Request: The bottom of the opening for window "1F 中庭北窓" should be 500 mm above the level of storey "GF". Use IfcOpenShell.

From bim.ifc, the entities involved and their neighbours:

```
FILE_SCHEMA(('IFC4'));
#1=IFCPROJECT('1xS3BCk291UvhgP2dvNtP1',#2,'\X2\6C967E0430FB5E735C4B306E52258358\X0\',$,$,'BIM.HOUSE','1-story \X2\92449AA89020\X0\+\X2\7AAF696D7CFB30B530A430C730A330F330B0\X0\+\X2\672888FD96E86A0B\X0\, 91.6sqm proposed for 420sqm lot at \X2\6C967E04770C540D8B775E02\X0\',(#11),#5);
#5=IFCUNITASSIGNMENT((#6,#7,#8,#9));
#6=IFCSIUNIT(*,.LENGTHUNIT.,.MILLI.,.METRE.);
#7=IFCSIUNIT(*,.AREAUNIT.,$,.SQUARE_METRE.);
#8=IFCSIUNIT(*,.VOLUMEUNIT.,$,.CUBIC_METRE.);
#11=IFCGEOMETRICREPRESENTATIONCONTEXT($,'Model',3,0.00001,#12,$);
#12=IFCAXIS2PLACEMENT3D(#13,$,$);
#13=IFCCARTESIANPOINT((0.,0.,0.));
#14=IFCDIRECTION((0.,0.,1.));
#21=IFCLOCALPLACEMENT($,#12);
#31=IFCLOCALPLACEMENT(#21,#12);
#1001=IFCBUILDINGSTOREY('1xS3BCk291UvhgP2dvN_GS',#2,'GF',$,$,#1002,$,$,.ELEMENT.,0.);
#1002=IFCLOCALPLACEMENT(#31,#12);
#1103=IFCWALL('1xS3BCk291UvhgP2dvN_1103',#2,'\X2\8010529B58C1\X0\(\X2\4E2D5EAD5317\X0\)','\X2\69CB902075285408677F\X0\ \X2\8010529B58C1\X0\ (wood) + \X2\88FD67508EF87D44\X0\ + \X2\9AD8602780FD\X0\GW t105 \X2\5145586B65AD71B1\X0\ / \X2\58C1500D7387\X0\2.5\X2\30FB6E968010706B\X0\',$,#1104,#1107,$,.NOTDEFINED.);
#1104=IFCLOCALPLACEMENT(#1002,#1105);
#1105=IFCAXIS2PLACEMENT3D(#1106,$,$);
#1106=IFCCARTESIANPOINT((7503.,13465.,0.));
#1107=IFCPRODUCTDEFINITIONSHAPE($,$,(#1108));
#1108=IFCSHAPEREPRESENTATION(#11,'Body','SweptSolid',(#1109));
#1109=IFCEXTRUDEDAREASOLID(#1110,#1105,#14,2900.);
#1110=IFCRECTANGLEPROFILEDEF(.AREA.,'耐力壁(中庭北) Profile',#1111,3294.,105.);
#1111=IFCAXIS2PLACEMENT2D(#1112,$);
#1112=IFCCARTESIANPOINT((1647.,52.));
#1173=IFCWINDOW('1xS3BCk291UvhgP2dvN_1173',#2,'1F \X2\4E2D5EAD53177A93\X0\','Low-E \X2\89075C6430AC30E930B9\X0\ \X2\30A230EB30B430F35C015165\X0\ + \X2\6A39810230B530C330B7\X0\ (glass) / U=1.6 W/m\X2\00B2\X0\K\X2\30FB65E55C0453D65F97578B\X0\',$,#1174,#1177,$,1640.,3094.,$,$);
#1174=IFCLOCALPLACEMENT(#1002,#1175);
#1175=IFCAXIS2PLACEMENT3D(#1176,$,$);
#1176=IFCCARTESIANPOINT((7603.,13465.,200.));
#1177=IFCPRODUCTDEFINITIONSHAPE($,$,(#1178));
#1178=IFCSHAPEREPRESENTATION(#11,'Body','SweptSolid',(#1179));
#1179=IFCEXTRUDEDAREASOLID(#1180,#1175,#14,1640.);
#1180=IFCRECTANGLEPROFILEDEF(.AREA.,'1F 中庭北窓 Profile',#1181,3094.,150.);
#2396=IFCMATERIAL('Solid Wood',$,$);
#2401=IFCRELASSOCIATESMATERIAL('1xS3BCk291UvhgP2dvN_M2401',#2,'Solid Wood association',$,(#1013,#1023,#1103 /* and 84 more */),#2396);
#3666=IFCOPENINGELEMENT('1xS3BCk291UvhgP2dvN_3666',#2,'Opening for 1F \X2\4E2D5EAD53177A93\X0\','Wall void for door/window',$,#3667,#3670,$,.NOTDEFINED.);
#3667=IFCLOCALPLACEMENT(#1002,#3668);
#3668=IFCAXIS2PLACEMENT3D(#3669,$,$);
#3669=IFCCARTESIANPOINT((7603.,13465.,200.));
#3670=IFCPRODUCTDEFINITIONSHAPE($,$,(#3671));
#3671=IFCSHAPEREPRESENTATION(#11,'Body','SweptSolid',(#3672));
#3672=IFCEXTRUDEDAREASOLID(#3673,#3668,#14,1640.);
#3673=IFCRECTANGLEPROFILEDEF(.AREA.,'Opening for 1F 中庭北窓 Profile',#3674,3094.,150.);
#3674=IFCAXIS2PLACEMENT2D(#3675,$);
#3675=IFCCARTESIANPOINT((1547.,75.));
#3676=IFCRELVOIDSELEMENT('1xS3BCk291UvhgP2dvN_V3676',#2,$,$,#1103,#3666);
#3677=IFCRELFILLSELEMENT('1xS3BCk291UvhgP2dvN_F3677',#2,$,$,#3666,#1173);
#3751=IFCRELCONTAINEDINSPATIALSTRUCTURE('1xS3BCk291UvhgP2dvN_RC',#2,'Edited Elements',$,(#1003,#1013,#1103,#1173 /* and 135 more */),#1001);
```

```python
import numpy as np
import ifcopenshell
import ifcopenshell.api.geometry
import ifcopenshell.geom
import ifcopenshell.util.element
import ifcopenshell.util.placement
import ifcopenshell.util.shape
import ifcopenshell.util.unit

model = ifcopenshell.open("bim.ifc")
unit_scale = ifcopenshell.util.unit.calculate_unit_scale(model)

window = model.by_guid("1xS3BCk291UvhgP2dvN_1173")
opening = window.FillsVoids[0].RelatingOpeningElement
storey = ifcopenshell.util.element.get_container(window, ifc_class="IfcBuildingStorey")
level = ifcopenshell.util.placement.get_local_placement(storey.ObjectPlacement)[2, 3]

# The opening's origin need not be at the sill, so measure its lowest point.
shape = ifcopenshell.geom.create_shape(ifcopenshell.geom.settings(), opening)
bottom = ifcopenshell.util.shape.get_shape_bottom_elevation(shape, shape.geometry) / unit_scale
dz = level + 500.0 - bottom

shift = np.array([0.0, 0.0, dz])
# The window is not placed relative to its opening, so move both.
for product in (opening, window):
    matrix = ifcopenshell.util.placement.get_local_placement(product.ObjectPlacement)
    matrix[:3, 3] += shift
    ifcopenshell.api.geometry.edit_object_placement(model, product=product, matrix=matrix, is_si=False)

print(f"moved by {dz * unit_scale:+.3f} m")

model.write("bim_edited.ifc")
```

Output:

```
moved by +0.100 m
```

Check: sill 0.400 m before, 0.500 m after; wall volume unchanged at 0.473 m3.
